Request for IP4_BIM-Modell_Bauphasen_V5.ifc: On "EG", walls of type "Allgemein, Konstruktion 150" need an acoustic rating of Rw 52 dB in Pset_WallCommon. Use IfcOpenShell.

First a look at what the model holds.

```python
import ifcopenshell
import ifcopenshell.util.element

model = ifcopenshell.open("IP4_BIM-Modell_Bauphasen_V5.ifc")
print(model.schema)
storey = next(s for s in model.by_type("IfcBuildingStorey") if s.Name == "EG")
walls = [e for e in ifcopenshell.util.element.get_decomposition(storey) if e.is_a("IfcWall")]
seen = {}
for e in walls:
    element_type = ifcopenshell.util.element.get_type(e)
    key = (element_type.Name if element_type != e and element_type else None, ifcopenshell.util.element.get_pset(e, "Pset_WallCommon", "AcousticRating"))
    seen[key] = seen.get(key, 0) + 1
for (name, value), count in sorted(seen.items(), key=str):
    print(count, "x", name, "|", value)
```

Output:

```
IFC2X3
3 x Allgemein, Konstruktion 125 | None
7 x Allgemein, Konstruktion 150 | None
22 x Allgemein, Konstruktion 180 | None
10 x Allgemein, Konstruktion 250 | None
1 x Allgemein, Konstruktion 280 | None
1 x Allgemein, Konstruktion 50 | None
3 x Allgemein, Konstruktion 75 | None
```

```python
import ifcopenshell
import ifcopenshell.api.pset
import ifcopenshell.util.element

model = ifcopenshell.open("IP4_BIM-Modell_Bauphasen_V5.ifc")

storey = next(s for s in model.by_type("IfcBuildingStorey") if s.Name == "EG")
walls = [e for e in ifcopenshell.util.element.get_decomposition(storey) if e.is_a("IfcWall")]

count = 0
for e in walls:
    element_type = ifcopenshell.util.element.get_type(e)
    if element_type in (None, e) or element_type.Name != "Allgemein, Konstruktion 150":
        continue
    # add_pset returns the element's existing set when there is one.
    pset = ifcopenshell.api.pset.add_pset(model, product=e, name="Pset_WallCommon")
    ifcopenshell.api.pset.edit_pset(model, pset=pset, properties={"AcousticRating": "Rw 52 dB"})
    count += 1

print(count, "walls updated")

model.write("IP4_BIM-Modell_Bauphasen_V5_rev.ifc")
```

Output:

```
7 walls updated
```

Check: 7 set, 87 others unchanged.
